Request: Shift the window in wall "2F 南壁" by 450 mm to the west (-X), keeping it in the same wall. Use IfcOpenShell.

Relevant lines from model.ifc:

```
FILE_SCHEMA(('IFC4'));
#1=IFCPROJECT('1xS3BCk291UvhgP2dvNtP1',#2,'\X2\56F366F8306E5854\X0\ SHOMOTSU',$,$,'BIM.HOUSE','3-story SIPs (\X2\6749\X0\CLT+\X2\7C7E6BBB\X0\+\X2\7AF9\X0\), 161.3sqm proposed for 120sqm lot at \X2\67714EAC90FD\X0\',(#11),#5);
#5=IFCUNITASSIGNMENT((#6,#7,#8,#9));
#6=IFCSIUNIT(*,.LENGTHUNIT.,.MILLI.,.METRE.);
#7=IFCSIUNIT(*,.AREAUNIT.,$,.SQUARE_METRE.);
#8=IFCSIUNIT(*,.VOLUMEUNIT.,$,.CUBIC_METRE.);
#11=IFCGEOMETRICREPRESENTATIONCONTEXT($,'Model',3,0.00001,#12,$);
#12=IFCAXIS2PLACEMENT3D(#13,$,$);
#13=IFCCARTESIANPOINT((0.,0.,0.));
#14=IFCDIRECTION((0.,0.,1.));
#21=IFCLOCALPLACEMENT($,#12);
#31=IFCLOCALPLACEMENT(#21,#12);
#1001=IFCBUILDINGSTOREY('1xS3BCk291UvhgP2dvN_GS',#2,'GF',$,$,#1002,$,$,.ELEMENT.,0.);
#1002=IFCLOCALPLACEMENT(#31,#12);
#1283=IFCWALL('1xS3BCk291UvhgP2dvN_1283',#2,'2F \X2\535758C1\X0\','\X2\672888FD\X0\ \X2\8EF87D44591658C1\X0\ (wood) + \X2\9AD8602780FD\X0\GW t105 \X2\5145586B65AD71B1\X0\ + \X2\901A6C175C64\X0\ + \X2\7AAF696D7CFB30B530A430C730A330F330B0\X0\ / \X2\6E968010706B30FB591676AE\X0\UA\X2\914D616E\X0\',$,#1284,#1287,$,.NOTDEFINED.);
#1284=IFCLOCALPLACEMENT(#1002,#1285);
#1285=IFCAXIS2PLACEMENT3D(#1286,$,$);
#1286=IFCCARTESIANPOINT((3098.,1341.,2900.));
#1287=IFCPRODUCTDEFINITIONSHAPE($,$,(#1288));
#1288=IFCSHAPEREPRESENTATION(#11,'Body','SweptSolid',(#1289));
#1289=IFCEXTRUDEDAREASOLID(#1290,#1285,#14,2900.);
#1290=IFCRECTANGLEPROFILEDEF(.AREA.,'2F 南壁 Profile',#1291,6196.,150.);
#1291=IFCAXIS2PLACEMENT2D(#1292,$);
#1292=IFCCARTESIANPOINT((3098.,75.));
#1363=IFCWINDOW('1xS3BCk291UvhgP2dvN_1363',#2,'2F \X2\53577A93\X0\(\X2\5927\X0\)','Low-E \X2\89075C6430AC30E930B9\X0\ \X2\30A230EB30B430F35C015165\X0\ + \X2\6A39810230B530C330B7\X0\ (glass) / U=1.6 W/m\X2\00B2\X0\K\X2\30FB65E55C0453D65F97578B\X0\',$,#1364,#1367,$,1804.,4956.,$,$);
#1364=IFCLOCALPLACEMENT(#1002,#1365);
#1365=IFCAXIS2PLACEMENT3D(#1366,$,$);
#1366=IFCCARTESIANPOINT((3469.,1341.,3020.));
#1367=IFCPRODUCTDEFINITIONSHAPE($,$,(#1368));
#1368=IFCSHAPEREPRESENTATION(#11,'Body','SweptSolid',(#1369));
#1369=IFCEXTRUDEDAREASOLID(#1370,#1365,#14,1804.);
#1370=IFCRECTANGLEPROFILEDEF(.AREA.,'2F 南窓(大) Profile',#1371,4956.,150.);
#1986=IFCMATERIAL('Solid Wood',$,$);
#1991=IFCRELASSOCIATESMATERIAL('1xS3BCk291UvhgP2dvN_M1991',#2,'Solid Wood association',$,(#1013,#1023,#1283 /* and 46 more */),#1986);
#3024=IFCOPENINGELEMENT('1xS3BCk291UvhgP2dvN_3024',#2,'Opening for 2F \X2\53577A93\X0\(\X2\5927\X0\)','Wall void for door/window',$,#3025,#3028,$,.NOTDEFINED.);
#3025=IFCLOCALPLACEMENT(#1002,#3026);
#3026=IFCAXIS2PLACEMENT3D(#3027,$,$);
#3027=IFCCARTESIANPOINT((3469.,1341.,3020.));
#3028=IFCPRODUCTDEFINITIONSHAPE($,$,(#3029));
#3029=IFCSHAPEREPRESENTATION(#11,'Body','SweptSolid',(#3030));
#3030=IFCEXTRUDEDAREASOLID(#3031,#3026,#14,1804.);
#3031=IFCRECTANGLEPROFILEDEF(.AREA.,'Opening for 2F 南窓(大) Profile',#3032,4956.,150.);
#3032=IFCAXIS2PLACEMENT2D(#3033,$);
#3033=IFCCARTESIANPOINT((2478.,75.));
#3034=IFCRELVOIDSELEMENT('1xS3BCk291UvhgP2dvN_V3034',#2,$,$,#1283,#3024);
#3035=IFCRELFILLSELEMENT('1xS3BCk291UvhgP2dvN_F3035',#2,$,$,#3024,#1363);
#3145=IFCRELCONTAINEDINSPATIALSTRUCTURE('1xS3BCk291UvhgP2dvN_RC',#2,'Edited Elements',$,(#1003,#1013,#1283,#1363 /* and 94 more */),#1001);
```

```python
import ifcopenshell
import ifcopenshell.api.geometry
import ifcopenshell.util.placement
import ifcopenshell.util.unit

model = ifcopenshell.open("model.ifc")
unit_scale = ifcopenshell.util.unit.calculate_unit_scale(model)

window = model.by_guid("1xS3BCk291UvhgP2dvN_1363")
opening = window.FillsVoids[0].RelatingOpeningElement
wall = opening.VoidsElements[0].RelatingBuildingElement

wall_matrix = ifcopenshell.util.placement.get_local_placement(wall.ObjectPlacement)
shift = wall_matrix[:3, 0] * -0.45 / unit_scale
before = ifcopenshell.util.placement.get_local_placement(window.ObjectPlacement)[:3, 3].copy()

# The window is not placed relative to its opening, so move both.
for product in (opening, window):
    matrix = ifcopenshell.util.placement.get_local_placement(product.ObjectPlacement)
    matrix[:3, 3] += shift
    ifcopenshell.api.geometry.edit_object_placement(model, product=product, matrix=matrix, is_si=False)

after = ifcopenshell.util.placement.get_local_placement(window.ObjectPlacement)[:3, 3]
print("window moved by", (after - before).round(3) + 0.0)

model.write("model_edited.ifc")
```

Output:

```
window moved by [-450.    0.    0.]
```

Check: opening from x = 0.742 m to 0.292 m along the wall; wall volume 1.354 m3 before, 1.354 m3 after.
